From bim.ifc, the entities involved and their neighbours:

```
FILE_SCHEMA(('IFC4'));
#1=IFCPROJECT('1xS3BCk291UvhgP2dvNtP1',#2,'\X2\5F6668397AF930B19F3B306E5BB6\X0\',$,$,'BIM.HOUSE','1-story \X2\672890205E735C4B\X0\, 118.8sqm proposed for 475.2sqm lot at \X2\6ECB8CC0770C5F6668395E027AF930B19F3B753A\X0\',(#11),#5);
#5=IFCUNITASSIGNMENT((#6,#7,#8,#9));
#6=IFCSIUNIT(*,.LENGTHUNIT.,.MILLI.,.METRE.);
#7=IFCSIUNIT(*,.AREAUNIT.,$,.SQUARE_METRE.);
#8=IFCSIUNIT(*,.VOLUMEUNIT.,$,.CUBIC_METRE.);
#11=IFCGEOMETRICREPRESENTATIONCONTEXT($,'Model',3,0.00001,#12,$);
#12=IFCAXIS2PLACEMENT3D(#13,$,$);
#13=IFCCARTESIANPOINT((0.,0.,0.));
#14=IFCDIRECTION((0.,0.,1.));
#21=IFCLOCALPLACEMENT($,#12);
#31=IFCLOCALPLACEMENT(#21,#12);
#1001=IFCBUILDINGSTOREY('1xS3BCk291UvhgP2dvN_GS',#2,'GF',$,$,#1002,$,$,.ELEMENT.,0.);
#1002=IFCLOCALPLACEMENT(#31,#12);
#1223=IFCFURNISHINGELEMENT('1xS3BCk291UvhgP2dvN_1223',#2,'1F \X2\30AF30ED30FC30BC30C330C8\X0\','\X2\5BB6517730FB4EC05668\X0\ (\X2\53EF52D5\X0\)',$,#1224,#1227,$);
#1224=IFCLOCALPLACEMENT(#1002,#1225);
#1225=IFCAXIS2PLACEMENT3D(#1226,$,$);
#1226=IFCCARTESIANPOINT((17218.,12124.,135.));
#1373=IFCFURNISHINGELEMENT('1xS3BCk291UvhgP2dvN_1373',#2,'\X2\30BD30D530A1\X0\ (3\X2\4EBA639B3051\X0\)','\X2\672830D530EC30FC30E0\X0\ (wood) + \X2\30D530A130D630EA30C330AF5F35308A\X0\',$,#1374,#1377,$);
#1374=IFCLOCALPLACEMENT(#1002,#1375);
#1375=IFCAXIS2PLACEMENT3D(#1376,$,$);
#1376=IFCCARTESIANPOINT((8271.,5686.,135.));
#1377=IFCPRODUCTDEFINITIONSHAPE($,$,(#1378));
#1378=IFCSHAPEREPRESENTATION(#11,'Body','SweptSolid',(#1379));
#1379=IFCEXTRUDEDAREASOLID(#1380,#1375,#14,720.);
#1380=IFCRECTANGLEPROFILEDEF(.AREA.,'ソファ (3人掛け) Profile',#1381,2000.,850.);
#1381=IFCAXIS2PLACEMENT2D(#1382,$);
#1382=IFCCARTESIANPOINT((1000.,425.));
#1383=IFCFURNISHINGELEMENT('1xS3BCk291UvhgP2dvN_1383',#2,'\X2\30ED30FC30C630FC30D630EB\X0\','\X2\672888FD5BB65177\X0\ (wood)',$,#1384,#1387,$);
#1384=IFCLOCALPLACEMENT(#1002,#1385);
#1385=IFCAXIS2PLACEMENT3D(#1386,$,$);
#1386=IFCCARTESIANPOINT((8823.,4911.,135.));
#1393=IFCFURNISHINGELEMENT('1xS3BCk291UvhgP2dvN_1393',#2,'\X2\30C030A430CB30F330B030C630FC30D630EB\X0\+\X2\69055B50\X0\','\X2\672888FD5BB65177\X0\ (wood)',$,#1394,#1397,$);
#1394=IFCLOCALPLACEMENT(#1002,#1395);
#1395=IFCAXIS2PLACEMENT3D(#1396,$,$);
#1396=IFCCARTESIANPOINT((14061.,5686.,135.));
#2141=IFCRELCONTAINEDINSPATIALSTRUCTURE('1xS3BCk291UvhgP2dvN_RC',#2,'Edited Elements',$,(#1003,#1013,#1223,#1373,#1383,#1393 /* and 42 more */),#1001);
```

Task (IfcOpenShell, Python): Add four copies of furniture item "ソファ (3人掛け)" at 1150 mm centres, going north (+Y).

```python
import numpy as np
import ifcopenshell
import ifcopenshell.api.geometry
import ifcopenshell.api.root
import ifcopenshell.util.element
import ifcopenshell.util.placement

model = ifcopenshell.open("bim.ifc")


def reuse_history(source, copy):
    """copy_class also copies each property set's owner history, people and application; keep the originals."""
    for rel in copy.IsDefinedBy:
        if rel.is_a("IfcRelDefinesByProperties") and (history := rel.RelatingPropertyDefinition.OwnerHistory):
            rel.RelatingPropertyDefinition.OwnerHistory = source.OwnerHistory
            ifcopenshell.util.element.remove_deep2(model, history)


source = model.by_id(1373)
base = ifcopenshell.util.placement.get_local_placement(source.ObjectPlacement)
step = np.array([0.0, 1.0, 0.0]) * 1150.0

for i in range(1, 5):
    copy = ifcopenshell.api.root.copy_class(model, product=source)
    copy.Representation = ifcopenshell.util.element.copy_deep(
        model, source.Representation, exclude=["IfcGeometricRepresentationContext", "IfcRepresentationMap"]
    )
    reuse_history(source, copy)
    matrix = base.copy()
    matrix[:3, 3] += i * step
    print("added at", matrix[:3, 3].round(3) + 0.0)
    ifcopenshell.api.geometry.edit_object_placement(model, product=copy, matrix=matrix, is_si=False)

model.write("bim_rev.ifc")
```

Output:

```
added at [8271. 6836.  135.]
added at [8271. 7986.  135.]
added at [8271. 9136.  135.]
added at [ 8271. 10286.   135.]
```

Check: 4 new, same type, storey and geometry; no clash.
